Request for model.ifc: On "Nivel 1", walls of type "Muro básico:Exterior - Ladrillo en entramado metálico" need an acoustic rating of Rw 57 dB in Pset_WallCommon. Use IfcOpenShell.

First a look at what the model holds.

```python
import ifcopenshell
import ifcopenshell.util.element

model = ifcopenshell.open("model.ifc")
print(model.schema)
storey = next(s for s in model.by_type("IfcBuildingStorey") if s.Name == "Nivel 1")
walls = [e for e in ifcopenshell.util.element.get_decomposition(storey) if e.is_a("IfcWall")]
seen = {}
for e in walls:
    element_type = ifcopenshell.util.element.get_type(e)
    key = (element_type.Name if element_type != e and element_type else None, ifcopenshell.util.element.get_pset(e, "Pset_WallCommon", "AcousticRating"))
    seen[key] = seen.get(key, 0) + 1
for (name, value), count in sorted(seen.items(), key=str):
    print(count, "x", name, "|", value)
```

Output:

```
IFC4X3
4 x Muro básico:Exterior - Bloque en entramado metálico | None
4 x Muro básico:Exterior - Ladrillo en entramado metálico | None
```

```python
import ifcopenshell
import ifcopenshell.api.pset
import ifcopenshell.util.element

model = ifcopenshell.open("model.ifc")

storey = next(s for s in model.by_type("IfcBuildingStorey") if s.Name == "Nivel 1")
walls = [e for e in ifcopenshell.util.element.get_decomposition(storey) if e.is_a("IfcWall")]

count = 0
for e in walls:
    element_type = ifcopenshell.util.element.get_type(e)
    if element_type in (None, e) or element_type.Name != "Muro básico:Exterior - Ladrillo en entramado metálico":
        continue
    # add_pset returns the element's existing set when there is one.
    pset = ifcopenshell.api.pset.add_pset(model, product=e, name="Pset_WallCommon")
    ifcopenshell.api.pset.edit_pset(model, pset=pset, properties={"AcousticRating": "Rw 57 dB"})
    count += 1

print(count, "walls updated")

model.write("model_rev.ifc")
```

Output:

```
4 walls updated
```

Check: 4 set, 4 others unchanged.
